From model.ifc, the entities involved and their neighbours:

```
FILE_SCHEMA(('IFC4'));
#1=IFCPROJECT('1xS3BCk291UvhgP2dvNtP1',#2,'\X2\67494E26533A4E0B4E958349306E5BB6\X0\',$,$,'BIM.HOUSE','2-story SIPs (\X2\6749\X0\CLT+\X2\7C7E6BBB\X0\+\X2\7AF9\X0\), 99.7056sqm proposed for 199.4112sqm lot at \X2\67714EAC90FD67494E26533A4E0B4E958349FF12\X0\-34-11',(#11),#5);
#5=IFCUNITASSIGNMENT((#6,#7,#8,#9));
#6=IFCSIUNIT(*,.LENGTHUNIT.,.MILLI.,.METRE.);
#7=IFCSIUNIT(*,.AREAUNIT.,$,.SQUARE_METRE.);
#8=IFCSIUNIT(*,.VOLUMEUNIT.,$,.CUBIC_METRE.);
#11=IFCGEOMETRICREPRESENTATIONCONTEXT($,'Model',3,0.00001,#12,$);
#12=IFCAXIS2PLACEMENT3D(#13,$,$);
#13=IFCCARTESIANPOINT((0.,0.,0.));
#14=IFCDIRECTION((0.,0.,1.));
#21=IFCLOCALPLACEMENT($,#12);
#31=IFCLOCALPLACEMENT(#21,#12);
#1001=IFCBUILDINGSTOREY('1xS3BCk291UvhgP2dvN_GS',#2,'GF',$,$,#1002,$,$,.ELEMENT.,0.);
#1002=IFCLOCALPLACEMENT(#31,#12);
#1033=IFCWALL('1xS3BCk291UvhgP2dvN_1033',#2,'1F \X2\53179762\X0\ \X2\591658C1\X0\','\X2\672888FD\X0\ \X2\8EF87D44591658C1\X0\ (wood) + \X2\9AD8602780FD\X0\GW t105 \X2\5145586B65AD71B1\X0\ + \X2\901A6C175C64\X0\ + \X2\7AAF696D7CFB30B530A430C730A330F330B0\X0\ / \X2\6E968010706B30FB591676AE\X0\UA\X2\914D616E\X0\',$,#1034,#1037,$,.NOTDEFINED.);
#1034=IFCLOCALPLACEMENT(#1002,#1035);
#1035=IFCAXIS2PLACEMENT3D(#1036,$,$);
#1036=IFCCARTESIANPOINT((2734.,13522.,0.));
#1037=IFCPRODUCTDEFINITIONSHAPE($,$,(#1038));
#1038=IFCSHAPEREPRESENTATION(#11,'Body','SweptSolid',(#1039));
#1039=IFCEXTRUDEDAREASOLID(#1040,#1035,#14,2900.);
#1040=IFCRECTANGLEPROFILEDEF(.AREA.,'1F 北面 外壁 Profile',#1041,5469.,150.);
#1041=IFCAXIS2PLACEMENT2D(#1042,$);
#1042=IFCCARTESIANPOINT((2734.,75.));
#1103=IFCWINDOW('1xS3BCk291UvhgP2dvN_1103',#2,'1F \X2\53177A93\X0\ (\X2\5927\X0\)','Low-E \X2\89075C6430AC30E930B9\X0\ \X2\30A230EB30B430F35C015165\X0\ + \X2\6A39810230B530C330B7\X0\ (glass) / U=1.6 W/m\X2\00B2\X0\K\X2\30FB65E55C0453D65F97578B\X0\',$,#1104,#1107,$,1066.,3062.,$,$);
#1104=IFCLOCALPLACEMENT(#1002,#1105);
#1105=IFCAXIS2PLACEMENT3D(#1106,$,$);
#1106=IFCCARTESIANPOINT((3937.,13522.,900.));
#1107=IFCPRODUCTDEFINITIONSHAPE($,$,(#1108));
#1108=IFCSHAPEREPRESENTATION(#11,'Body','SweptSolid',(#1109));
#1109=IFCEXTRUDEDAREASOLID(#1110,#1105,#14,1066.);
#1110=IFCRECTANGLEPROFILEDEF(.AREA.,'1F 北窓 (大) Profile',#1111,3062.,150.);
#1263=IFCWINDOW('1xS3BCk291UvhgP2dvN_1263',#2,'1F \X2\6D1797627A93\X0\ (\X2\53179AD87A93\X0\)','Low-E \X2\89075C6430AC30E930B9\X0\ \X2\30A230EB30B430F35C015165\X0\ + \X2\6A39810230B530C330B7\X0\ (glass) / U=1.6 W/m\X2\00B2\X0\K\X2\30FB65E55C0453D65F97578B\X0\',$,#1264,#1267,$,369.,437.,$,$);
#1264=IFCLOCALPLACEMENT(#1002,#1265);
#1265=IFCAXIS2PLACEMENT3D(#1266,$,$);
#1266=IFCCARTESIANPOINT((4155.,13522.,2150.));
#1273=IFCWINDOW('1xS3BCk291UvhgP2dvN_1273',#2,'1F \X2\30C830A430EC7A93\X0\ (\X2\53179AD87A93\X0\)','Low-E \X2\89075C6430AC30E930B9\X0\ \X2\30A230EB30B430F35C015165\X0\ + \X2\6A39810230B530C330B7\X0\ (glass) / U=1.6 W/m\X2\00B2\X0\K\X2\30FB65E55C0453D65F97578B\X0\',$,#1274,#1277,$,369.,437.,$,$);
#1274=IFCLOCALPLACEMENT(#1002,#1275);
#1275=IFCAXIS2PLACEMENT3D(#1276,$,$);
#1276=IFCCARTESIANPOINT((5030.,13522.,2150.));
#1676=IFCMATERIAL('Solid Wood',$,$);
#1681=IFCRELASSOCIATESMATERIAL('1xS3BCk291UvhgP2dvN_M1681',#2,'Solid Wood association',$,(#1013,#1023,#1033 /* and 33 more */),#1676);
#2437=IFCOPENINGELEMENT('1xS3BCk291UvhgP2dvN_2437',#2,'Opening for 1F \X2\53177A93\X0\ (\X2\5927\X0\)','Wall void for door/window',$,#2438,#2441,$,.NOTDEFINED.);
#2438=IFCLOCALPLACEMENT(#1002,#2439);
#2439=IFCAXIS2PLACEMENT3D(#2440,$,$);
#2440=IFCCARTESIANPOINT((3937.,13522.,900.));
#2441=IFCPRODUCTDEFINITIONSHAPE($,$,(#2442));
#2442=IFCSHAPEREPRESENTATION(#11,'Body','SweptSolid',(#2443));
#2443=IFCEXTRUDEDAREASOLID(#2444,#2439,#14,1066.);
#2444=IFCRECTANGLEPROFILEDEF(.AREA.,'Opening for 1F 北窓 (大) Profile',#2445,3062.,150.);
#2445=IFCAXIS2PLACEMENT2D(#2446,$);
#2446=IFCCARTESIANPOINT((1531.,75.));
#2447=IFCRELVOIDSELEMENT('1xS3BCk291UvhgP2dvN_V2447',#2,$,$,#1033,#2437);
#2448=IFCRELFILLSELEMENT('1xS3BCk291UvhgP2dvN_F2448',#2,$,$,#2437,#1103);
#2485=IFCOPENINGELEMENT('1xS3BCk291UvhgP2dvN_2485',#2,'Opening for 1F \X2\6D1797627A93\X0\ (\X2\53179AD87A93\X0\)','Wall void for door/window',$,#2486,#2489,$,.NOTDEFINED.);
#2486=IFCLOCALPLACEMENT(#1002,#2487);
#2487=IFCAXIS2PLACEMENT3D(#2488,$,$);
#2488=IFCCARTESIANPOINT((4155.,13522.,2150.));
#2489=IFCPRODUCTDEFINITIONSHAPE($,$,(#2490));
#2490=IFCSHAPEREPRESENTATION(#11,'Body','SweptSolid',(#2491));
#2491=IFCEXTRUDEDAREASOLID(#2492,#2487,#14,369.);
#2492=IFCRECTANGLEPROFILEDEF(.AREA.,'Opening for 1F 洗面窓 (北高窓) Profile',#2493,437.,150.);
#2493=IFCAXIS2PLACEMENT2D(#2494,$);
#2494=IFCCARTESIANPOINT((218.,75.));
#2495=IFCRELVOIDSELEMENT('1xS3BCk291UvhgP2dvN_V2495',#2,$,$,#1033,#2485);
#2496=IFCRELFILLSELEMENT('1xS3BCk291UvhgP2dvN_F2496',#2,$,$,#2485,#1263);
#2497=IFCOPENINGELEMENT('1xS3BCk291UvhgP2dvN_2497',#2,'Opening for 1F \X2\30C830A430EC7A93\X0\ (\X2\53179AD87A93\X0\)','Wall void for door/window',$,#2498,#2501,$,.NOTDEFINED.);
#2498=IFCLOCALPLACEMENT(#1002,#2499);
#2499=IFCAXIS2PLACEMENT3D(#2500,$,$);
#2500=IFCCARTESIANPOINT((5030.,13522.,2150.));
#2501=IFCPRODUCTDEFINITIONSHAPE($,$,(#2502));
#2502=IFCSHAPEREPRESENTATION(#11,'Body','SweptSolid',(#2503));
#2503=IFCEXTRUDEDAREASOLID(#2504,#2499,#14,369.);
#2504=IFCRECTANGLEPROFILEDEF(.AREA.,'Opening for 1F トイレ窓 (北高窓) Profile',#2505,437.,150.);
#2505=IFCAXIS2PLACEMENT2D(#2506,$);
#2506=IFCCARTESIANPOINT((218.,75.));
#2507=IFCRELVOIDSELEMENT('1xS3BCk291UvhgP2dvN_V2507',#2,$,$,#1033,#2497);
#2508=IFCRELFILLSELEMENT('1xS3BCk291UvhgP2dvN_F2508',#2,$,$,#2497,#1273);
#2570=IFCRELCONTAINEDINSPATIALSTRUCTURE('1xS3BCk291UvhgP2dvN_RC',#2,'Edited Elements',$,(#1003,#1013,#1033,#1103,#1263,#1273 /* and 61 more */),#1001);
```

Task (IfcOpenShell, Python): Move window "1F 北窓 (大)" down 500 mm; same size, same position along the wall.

```python
import numpy as np
import ifcopenshell
import ifcopenshell.api.geometry
import ifcopenshell.util.placement
import ifcopenshell.util.unit

model = ifcopenshell.open("model.ifc")
unit_scale = ifcopenshell.util.unit.calculate_unit_scale(model)

window = model.by_id(1103)
opening = window.FillsVoids[0].RelatingOpeningElement
dz = -0.5 / unit_scale

shift = np.array([0.0, 0.0, dz])
# The window is not placed relative to its opening, so move both.
for product in (opening, window):
    matrix = ifcopenshell.util.placement.get_local_placement(product.ObjectPlacement)
    matrix[:3, 3] += shift
    ifcopenshell.api.geometry.edit_object_placement(model, product=product, matrix=matrix, is_si=False)

print(f"moved by {dz * unit_scale:+.3f} m")

model.write("model_edited.ifc")
```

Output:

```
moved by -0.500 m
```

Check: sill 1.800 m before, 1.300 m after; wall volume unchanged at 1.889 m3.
